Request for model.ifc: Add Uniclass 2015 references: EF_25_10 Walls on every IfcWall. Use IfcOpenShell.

First a look at what the model holds.

```python
import ifcopenshell

model = ifcopenshell.open("model.ifc")
print(model.schema)
print("classifications:", [c.Name for c in model.by_type("IfcClassification")])
for ifc_class in ("IfcDoor", "IfcRoof", "IfcStair", "IfcWall", "IfcWindow"):
    print(ifc_class, len(model.by_type(ifc_class)))
```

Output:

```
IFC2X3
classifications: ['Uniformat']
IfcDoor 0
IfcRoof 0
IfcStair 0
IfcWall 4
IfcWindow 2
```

```python
import ifcopenshell
import ifcopenshell.api.classification

model = ifcopenshell.open("model.ifc")

# IFC2X3 requires Source and Edition and has no link from the project to the system.
system = model.create_entity("IfcClassification", Source="NBS", Edition="2015", Name="Uniclass 2015")

codes = {
    "IfcWall": ("EF_25_10", "Walls"),
}
for ifc_class, (code, name) in codes.items():
    products = model.by_type(ifc_class)
    ifcopenshell.api.classification.add_reference(
        model, products=products, classification=system, identification=code, name=name
    )
    print(code, len(products))

model.write("model_rev.ifc")
```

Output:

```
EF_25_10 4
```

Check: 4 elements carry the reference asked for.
